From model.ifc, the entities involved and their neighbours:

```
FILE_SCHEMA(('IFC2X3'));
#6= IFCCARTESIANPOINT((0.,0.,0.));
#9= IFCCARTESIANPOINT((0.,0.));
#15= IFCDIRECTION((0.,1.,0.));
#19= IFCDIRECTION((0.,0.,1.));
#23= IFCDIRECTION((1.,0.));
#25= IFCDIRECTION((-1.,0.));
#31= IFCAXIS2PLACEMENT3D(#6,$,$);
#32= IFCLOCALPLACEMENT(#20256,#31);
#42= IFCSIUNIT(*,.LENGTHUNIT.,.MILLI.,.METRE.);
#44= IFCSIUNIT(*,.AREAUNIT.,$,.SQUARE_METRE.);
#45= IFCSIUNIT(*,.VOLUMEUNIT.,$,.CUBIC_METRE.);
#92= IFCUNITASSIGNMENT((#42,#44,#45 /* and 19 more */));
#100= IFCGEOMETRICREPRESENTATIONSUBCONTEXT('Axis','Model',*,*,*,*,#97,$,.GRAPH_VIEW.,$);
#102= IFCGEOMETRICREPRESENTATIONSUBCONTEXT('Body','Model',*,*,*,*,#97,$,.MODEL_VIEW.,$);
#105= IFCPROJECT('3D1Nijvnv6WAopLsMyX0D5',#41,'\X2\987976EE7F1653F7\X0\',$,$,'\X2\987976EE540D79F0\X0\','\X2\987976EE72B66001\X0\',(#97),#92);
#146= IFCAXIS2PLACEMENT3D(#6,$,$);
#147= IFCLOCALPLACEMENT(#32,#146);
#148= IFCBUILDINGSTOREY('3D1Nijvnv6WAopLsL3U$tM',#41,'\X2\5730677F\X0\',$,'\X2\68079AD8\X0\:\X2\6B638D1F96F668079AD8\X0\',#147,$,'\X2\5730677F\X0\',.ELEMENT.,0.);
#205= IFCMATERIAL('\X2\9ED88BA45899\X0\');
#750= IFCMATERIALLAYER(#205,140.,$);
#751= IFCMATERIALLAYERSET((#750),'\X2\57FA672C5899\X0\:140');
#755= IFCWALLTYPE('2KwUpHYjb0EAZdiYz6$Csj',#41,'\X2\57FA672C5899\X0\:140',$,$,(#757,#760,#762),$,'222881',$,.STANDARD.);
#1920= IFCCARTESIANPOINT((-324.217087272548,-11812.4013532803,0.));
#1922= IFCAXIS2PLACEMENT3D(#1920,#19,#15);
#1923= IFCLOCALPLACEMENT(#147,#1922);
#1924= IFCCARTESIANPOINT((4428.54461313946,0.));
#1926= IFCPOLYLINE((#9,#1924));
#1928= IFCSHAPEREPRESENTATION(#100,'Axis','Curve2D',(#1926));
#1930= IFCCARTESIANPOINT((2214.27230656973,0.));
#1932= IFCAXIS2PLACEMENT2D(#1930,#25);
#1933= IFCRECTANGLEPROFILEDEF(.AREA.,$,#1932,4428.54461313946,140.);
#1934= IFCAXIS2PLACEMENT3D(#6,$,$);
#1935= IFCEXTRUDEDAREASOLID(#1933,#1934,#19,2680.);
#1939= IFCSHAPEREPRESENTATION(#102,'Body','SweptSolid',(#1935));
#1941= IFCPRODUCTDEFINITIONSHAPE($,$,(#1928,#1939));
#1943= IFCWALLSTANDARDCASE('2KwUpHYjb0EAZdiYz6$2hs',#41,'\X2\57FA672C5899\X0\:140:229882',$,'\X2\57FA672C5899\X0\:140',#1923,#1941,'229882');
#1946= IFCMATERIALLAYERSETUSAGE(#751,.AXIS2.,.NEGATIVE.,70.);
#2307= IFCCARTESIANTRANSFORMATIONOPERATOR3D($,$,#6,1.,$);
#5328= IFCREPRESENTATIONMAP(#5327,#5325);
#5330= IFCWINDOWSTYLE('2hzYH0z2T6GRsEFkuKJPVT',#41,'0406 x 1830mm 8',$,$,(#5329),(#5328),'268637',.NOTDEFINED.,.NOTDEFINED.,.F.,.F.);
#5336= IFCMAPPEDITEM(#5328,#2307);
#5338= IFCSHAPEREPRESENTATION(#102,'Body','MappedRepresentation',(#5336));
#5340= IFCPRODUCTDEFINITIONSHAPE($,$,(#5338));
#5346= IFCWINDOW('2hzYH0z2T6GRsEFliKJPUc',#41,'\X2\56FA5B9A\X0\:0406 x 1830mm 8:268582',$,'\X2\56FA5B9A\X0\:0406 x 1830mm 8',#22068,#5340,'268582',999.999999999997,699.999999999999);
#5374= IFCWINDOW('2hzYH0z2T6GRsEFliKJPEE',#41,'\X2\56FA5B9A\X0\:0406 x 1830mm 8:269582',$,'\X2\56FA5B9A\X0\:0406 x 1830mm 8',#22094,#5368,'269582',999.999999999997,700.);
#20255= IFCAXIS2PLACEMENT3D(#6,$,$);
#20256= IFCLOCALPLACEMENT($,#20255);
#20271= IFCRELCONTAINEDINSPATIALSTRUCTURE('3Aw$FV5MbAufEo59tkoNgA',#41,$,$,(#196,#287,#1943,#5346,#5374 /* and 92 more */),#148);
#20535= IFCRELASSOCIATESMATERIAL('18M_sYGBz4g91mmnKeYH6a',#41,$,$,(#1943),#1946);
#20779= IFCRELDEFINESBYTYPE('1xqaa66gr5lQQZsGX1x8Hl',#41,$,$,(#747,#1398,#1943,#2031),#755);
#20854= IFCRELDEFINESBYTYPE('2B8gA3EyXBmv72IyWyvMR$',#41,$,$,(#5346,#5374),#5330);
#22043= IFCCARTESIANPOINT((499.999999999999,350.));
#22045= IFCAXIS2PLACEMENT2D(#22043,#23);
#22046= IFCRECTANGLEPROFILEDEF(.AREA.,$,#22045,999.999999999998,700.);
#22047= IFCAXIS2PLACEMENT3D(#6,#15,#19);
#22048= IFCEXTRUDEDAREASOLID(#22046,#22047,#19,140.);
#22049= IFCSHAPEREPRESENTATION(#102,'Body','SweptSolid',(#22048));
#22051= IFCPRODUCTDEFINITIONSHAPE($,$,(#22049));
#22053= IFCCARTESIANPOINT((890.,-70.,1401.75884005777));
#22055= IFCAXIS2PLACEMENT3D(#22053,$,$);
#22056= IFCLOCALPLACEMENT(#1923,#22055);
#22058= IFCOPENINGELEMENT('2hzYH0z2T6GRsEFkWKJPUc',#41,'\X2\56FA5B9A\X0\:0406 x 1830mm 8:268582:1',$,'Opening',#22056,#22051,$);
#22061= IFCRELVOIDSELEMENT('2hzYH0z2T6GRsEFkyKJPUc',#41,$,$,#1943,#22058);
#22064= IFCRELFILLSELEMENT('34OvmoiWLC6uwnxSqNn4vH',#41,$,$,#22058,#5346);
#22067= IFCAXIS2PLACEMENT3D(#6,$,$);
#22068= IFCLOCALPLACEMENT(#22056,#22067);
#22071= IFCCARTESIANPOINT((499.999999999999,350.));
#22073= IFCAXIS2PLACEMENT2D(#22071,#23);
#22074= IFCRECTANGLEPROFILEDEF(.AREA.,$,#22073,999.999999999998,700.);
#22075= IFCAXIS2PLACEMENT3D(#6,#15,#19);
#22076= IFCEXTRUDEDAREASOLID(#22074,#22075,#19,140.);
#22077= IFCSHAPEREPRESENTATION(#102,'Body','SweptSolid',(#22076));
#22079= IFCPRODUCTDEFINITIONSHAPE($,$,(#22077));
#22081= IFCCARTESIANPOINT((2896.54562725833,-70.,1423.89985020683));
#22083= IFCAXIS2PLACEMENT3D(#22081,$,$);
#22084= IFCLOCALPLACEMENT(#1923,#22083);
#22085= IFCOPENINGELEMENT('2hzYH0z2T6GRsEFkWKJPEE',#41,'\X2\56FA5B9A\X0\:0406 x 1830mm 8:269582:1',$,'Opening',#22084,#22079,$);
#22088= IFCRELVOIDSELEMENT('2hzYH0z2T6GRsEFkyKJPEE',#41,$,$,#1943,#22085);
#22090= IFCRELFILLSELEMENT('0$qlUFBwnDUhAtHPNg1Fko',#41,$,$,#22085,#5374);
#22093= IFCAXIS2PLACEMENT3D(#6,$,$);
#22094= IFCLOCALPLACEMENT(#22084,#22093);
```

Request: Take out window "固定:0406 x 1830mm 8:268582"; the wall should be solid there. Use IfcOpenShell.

```python
import ifcopenshell
import ifcopenshell.api.feature
import ifcopenshell.api.root
import ifcopenshell.geom
import ifcopenshell.util.shape

model = ifcopenshell.open("model.ifc")
settings = ifcopenshell.geom.settings()


def volume(element):
    """Net volume in cubic metres, openings subtracted."""
    shape = ifcopenshell.geom.create_shape(settings, element)
    return ifcopenshell.util.shape.get_volume(shape.geometry)


window = model.by_id(5346)
opening = window.FillsVoids[0].RelatingOpeningElement
wall = opening.VoidsElements[0].RelatingBuildingElement
before = volume(wall)

ifcopenshell.api.root.remove_product(model, product=window)
ifcopenshell.api.feature.remove_feature(model, feature=opening)

after = volume(wall)

print(f"wall volume {before:.3f} -> {after:.3f} m3")

model.write("model_updated.ifc")
```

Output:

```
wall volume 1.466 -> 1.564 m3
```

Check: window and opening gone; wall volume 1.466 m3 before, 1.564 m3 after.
